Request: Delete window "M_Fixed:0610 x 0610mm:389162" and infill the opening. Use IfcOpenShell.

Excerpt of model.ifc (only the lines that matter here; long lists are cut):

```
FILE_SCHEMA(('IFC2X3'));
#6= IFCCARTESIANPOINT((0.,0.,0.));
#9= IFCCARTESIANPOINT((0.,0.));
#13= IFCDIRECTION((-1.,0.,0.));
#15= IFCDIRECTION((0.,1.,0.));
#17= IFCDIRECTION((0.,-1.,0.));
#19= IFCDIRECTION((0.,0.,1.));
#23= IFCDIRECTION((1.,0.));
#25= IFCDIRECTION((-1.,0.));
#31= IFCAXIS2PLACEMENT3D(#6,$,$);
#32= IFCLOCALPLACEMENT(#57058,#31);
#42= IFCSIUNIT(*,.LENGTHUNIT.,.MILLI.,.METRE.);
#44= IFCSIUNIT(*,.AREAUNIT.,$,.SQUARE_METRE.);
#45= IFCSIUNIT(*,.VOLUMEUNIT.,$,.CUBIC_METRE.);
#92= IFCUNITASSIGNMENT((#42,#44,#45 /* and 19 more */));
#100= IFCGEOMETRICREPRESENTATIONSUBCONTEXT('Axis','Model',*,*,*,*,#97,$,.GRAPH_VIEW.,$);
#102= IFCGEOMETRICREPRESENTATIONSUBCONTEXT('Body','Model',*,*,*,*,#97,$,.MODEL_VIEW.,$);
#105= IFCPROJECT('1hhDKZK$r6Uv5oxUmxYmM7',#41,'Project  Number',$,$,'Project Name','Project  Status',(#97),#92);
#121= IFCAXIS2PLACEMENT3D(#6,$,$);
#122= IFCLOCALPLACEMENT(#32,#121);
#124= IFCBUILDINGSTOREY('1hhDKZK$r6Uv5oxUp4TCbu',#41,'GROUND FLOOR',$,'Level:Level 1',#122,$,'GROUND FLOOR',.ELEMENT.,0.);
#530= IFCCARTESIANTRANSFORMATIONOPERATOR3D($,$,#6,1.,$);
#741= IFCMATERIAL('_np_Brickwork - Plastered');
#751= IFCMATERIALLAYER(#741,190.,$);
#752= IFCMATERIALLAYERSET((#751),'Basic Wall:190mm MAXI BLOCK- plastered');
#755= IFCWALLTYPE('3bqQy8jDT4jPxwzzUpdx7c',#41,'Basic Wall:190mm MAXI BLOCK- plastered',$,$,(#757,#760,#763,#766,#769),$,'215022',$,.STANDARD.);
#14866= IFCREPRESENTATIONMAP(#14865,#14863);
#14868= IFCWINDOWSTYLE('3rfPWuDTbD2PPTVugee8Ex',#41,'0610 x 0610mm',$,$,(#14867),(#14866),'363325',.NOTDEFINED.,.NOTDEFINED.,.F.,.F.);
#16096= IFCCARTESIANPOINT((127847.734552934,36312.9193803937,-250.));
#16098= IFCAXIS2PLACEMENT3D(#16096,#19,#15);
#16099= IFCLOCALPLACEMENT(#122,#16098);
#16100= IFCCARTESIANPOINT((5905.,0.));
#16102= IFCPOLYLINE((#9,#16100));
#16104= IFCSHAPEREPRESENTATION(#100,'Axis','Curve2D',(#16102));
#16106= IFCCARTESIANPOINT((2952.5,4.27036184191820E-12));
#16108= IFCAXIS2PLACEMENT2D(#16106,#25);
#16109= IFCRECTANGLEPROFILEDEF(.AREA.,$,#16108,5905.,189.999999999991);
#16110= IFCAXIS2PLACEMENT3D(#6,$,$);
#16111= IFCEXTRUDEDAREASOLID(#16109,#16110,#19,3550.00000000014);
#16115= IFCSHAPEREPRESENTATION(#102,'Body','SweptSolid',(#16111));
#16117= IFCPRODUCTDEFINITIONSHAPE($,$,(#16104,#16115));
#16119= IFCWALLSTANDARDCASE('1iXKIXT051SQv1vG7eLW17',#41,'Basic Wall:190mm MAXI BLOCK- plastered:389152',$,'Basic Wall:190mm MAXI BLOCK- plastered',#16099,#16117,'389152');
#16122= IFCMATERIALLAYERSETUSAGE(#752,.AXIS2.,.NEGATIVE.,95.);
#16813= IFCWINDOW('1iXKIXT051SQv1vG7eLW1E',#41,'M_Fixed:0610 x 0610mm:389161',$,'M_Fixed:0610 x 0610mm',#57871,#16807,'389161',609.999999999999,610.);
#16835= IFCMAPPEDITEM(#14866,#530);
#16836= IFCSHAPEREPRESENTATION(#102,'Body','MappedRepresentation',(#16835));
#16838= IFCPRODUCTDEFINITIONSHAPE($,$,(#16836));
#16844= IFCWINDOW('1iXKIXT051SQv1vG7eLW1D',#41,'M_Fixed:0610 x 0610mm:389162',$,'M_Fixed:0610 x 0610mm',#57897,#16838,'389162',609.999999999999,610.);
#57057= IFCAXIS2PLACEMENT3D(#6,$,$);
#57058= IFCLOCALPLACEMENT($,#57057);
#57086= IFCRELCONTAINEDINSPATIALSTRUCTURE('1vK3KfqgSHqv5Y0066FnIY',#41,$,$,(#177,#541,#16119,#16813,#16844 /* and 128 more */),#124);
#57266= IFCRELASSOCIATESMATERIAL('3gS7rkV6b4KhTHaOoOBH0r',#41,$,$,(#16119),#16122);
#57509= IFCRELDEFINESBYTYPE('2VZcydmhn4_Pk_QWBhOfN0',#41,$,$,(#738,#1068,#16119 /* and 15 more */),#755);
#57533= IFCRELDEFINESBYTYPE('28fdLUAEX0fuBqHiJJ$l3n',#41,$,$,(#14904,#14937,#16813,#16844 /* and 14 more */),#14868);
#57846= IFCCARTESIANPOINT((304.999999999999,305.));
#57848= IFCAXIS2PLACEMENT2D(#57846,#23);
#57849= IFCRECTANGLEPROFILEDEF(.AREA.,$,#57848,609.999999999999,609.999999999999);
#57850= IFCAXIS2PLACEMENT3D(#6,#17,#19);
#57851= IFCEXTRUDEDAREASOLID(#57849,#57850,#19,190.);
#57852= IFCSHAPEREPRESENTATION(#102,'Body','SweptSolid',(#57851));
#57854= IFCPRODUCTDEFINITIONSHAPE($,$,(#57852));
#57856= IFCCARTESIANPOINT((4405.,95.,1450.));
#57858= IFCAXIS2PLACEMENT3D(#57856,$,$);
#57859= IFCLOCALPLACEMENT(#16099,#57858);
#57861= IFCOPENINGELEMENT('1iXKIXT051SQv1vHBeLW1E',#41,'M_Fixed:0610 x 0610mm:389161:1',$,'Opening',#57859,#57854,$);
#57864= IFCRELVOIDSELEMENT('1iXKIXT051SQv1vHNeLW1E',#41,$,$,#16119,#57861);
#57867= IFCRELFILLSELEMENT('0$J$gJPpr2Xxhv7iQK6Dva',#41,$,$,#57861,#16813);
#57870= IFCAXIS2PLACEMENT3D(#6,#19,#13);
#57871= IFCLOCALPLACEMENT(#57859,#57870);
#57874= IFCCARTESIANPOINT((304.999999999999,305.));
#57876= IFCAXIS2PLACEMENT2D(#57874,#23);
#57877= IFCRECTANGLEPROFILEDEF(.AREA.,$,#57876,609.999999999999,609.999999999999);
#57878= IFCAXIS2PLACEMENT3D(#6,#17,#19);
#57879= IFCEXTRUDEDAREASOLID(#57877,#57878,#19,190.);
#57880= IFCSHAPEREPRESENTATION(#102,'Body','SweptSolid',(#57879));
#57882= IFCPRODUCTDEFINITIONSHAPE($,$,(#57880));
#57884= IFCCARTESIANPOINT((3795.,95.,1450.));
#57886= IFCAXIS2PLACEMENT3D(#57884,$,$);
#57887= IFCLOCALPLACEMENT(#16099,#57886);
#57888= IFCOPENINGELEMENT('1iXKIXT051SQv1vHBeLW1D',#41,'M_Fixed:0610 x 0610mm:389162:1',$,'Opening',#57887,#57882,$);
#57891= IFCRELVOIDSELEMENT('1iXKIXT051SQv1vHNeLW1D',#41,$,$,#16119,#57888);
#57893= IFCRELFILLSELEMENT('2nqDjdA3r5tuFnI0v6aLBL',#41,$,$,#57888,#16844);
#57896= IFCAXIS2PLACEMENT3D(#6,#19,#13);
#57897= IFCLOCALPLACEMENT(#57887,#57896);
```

```python
import ifcopenshell
import ifcopenshell.api.feature
import ifcopenshell.api.root
import ifcopenshell.geom
import ifcopenshell.util.shape

model = ifcopenshell.open("model.ifc")
settings = ifcopenshell.geom.settings()


def volume(element):
    """Net volume in cubic metres, openings subtracted."""
    shape = ifcopenshell.geom.create_shape(settings, element)
    return ifcopenshell.util.shape.get_volume(shape.geometry)


window = model.by_id(16844)
opening = window.FillsVoids[0].RelatingOpeningElement
wall = opening.VoidsElements[0].RelatingBuildingElement
before = volume(wall)

ifcopenshell.api.root.remove_product(model, product=window)
ifcopenshell.api.feature.remove_feature(model, feature=opening)

after = volume(wall)

print(f"wall volume {before:.3f} -> {after:.3f} m3")

model.write("model_rev.ifc")
```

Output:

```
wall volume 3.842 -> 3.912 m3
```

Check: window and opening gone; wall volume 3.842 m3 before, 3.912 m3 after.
